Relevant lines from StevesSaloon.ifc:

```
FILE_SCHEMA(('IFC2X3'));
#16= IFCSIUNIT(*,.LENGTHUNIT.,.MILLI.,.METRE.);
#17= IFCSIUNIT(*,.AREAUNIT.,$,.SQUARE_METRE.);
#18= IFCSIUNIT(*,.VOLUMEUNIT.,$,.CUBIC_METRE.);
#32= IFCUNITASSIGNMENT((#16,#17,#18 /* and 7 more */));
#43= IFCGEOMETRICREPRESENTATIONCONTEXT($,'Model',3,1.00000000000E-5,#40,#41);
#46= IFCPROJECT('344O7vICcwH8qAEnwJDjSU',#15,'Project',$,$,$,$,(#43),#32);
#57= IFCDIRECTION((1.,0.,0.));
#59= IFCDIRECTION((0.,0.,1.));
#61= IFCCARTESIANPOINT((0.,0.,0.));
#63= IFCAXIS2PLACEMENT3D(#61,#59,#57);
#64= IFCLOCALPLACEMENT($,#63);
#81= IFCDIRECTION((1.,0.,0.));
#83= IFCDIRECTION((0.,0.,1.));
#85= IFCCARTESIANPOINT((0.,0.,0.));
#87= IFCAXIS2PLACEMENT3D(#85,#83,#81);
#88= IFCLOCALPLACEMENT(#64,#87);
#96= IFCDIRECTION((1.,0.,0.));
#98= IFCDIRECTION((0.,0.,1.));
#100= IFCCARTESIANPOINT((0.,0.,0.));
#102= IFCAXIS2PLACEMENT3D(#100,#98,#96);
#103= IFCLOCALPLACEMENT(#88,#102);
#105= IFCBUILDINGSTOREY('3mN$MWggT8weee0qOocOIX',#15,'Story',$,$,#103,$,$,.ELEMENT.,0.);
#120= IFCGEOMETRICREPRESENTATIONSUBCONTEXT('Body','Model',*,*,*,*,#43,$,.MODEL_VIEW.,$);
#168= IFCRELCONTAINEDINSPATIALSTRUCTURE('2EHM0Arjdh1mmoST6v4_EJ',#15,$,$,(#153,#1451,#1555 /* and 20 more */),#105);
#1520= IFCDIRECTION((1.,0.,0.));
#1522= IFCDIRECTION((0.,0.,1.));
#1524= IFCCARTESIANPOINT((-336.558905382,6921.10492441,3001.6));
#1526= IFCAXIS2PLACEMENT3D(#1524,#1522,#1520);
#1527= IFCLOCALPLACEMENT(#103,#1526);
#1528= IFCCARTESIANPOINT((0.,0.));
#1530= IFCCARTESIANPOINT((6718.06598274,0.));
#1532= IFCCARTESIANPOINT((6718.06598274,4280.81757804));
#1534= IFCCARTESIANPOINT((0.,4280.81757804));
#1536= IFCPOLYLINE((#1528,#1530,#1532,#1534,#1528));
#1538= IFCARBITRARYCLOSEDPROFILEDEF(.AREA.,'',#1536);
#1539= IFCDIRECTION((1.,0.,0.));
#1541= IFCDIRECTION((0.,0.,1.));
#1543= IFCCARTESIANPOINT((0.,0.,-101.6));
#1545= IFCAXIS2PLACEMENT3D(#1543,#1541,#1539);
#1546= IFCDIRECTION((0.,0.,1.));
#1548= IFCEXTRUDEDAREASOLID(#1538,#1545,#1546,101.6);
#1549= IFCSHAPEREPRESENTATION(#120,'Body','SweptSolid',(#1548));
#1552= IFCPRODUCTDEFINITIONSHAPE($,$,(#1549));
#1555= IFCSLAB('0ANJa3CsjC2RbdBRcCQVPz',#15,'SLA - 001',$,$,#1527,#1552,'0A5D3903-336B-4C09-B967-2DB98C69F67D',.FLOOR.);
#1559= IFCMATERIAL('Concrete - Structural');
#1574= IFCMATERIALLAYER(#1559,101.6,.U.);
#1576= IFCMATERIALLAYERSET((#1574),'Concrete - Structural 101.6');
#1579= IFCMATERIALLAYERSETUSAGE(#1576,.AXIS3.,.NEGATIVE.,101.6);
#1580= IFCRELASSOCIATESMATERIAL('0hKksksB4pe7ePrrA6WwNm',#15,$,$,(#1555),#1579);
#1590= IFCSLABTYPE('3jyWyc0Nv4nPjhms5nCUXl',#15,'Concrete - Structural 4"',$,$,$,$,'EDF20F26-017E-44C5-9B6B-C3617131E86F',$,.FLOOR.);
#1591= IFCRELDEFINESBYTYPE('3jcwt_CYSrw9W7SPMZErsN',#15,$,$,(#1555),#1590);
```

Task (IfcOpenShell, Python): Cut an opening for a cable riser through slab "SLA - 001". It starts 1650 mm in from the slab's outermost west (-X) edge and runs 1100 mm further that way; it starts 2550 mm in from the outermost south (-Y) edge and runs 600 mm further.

```python
import numpy as np
import ifcopenshell
import ifcopenshell.api.feature
import ifcopenshell.api.geometry
import ifcopenshell.api.root
import ifcopenshell.geom
import ifcopenshell.util.placement
import ifcopenshell.util.representation
import ifcopenshell.util.shape
import ifcopenshell.util.unit

model = ifcopenshell.open("StevesSaloon.ifc")
unit_scale = ifcopenshell.util.unit.calculate_unit_scale(model)
settings = ifcopenshell.geom.settings()


def volume(element):
    """Net volume in cubic metres, openings subtracted."""
    shape = ifcopenshell.geom.create_shape(settings, element)
    return ifcopenshell.util.shape.get_volume(shape.geometry)


slab = model.by_guid("0ANJa3CsjC2RbdBRcCQVPz")
before = volume(slab)

# Extent in the slab's own axes, in metres. The edges named are its -X and -Y sides.
slab_shape = ifcopenshell.geom.create_shape(settings, slab)
vertices = ifcopenshell.util.shape.get_vertices(slab_shape.geometry)
x_min, y_min, bottom = vertices.min(axis=0)
top = vertices[:, 2].max()

opening = ifcopenshell.api.root.create_entity(model, ifc_class="IfcOpeningElement", name="Cable riser opening")
context = ifcopenshell.util.representation.get_context(model, "Model", "Body", "MODEL_VIEW")
width, depth = 1.1, 0.6
outline = [(0.0, 0.0), (width, 0.0), (width, depth), (0.0, depth), (0.0, 0.0)]
# Overshoot both faces by 50 mm so the cut is clean.
shape = ifcopenshell.api.geometry.add_slab_representation(
    model, context=context, depth=top - bottom + 0.1, polyline=outline
)
ifcopenshell.api.geometry.assign_representation(model, product=opening, representation=shape)

matrix = ifcopenshell.util.placement.get_local_placement(slab.ObjectPlacement)
matrix[:, 3] = matrix @ np.append(np.array([x_min + 1.65, y_min + 2.55, bottom - 0.05]) / unit_scale, 1.0)
ifcopenshell.api.geometry.edit_object_placement(model, product=opening, matrix=matrix, is_si=False)
ifcopenshell.api.feature.add_feature(model, feature=opening, element=slab)

after = volume(slab)

print(f"slab volume {before:.3f} -> {after:.3f} m3")

model.write("StevesSaloon_updated.ifc")
```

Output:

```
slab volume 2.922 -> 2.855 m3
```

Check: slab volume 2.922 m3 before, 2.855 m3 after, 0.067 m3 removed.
